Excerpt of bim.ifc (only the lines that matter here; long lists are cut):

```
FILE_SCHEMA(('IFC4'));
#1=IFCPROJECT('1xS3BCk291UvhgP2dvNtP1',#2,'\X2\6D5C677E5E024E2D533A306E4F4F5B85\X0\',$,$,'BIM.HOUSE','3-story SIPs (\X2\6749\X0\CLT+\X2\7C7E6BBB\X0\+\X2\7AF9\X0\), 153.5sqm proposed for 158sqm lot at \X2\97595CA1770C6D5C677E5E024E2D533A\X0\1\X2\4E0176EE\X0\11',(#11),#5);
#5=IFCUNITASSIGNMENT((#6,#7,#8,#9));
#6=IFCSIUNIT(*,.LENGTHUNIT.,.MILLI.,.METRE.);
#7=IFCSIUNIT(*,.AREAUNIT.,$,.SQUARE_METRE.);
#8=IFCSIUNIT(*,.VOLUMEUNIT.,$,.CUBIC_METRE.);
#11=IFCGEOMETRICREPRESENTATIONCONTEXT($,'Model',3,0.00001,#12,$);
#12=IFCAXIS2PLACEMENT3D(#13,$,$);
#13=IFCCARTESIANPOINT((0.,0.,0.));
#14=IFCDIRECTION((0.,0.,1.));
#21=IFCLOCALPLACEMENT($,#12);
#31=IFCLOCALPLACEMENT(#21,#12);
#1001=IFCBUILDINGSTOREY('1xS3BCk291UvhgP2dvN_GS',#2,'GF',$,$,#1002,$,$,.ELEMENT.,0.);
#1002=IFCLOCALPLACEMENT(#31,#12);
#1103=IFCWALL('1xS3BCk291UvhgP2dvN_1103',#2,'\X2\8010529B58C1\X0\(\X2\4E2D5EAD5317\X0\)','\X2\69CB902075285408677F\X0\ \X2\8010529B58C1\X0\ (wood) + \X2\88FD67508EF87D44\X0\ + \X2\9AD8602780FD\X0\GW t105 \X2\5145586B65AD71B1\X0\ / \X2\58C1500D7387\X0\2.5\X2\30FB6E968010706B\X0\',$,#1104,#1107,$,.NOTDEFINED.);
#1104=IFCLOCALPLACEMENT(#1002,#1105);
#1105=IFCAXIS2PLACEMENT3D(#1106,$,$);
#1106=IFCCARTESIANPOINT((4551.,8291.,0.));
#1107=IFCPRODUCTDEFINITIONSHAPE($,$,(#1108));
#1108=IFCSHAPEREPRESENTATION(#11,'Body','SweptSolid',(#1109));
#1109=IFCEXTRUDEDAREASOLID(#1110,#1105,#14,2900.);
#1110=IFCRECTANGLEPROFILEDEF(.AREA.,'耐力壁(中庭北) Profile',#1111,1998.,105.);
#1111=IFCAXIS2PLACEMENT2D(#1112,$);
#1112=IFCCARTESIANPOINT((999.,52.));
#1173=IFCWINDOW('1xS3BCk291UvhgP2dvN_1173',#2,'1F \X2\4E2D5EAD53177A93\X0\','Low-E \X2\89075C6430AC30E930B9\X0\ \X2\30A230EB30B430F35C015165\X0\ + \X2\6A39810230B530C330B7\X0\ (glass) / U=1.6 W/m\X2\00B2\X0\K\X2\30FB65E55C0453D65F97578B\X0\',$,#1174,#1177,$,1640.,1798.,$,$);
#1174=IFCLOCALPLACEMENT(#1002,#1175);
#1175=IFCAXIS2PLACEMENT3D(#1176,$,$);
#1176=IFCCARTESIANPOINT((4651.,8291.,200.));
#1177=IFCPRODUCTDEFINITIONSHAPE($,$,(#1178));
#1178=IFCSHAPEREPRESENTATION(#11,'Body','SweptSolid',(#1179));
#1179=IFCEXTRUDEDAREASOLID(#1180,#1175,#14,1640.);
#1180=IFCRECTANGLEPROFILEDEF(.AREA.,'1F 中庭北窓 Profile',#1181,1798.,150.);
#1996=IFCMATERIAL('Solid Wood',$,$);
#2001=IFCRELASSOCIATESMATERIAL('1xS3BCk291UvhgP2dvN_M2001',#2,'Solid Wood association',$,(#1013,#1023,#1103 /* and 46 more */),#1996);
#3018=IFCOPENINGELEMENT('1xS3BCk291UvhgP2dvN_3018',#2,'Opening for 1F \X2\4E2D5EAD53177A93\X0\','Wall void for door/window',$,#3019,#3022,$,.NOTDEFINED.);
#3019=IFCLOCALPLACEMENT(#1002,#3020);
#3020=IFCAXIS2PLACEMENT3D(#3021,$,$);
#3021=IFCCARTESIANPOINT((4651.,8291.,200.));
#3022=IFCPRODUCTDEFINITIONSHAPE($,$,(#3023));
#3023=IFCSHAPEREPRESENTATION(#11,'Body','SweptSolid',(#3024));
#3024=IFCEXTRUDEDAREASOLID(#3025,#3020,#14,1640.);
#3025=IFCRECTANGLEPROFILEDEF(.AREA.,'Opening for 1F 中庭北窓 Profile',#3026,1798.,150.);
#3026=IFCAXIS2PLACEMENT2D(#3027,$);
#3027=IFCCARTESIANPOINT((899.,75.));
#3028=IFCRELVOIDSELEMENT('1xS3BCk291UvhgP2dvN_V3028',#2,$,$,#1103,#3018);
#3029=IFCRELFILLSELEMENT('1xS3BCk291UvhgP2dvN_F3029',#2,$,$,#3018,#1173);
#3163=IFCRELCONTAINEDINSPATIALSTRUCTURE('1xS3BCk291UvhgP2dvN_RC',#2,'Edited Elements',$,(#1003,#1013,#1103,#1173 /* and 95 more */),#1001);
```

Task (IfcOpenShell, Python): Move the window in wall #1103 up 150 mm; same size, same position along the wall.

```python
import numpy as np
import ifcopenshell
import ifcopenshell.api.geometry
import ifcopenshell.util.placement
import ifcopenshell.util.unit

model = ifcopenshell.open("bim.ifc")
unit_scale = ifcopenshell.util.unit.calculate_unit_scale(model)

window = model.by_guid("1xS3BCk291UvhgP2dvN_1173")
opening = window.FillsVoids[0].RelatingOpeningElement
dz = 0.15 / unit_scale

shift = np.array([0.0, 0.0, dz])
# The window is not placed relative to its opening, so move both.
for product in (opening, window):
    matrix = ifcopenshell.util.placement.get_local_placement(product.ObjectPlacement)
    matrix[:3, 3] += shift
    ifcopenshell.api.geometry.edit_object_placement(model, product=product, matrix=matrix, is_si=False)

print(f"moved by {dz * unit_scale:+.3f} m")

model.write("bim_v2.ifc")
```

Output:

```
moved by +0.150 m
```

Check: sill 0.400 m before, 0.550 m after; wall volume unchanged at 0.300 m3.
